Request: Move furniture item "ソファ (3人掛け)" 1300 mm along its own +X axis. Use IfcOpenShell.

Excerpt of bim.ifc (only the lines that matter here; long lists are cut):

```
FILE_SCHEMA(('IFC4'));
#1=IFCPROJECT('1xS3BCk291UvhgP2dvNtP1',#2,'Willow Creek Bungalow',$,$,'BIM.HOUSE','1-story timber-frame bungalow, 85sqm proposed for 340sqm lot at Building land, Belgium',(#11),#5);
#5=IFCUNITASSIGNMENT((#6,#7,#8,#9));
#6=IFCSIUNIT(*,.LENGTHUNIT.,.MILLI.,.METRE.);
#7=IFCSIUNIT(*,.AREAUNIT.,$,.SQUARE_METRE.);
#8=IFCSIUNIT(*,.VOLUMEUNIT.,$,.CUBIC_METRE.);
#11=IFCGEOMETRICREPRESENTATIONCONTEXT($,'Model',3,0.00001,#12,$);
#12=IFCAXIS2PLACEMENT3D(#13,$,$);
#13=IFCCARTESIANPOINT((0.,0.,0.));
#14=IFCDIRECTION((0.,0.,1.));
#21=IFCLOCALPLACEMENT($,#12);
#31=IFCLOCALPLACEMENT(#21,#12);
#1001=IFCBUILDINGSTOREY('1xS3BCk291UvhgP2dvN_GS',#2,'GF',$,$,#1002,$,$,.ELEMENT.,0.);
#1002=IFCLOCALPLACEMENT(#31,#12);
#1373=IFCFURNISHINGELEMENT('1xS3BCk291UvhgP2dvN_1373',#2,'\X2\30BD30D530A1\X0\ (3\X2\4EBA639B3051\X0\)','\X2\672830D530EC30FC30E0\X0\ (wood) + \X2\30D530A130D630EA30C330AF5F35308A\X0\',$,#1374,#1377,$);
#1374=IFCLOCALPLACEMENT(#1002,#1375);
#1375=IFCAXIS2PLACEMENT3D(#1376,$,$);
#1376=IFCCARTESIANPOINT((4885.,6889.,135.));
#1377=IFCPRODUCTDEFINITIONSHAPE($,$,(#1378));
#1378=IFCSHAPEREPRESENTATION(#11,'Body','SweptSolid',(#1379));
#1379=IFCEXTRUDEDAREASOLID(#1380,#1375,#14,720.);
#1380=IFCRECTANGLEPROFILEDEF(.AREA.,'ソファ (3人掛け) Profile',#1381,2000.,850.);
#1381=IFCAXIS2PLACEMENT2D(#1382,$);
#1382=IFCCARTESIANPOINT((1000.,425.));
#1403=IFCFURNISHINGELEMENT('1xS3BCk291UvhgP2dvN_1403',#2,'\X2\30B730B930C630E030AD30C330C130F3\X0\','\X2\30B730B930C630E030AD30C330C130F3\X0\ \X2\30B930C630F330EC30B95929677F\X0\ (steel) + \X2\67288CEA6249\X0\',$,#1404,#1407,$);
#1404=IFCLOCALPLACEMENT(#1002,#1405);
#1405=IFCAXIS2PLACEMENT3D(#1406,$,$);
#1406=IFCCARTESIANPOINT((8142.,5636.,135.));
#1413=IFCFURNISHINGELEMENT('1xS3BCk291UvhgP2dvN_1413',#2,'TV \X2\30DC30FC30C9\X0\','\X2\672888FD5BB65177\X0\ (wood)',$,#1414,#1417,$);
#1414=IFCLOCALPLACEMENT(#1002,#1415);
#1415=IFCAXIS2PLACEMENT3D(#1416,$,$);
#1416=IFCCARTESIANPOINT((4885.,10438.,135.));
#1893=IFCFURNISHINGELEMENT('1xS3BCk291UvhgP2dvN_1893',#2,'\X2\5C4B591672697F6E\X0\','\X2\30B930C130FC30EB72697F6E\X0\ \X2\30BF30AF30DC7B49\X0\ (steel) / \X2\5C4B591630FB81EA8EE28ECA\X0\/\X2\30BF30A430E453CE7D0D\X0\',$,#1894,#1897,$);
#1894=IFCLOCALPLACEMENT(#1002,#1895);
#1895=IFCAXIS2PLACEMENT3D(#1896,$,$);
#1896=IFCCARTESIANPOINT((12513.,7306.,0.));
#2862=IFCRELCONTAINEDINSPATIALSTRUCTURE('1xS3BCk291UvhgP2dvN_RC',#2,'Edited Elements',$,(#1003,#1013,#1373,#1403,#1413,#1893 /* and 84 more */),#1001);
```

```python
import ifcopenshell
import ifcopenshell.api.geometry
import ifcopenshell.util.placement
import ifcopenshell.util.unit

model = ifcopenshell.open("bim.ifc")
unit_scale = ifcopenshell.util.unit.calculate_unit_scale(model)

item = model.by_id(1373)
matrix = ifcopenshell.util.placement.get_local_placement(item.ObjectPlacement)
matrix[:3, 3] += matrix[:3, 0] * 1.3 / unit_scale
ifcopenshell.api.geometry.edit_object_placement(model, product=item, matrix=matrix, is_si=False)

print(ifcopenshell.util.placement.get_local_placement(item.ObjectPlacement).round(3) + 0.0)

model.write("bim_edited.ifc")
```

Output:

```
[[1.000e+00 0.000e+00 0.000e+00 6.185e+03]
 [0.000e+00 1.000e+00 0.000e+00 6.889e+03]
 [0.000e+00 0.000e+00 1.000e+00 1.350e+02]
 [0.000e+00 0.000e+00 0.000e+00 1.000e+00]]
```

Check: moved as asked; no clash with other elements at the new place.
